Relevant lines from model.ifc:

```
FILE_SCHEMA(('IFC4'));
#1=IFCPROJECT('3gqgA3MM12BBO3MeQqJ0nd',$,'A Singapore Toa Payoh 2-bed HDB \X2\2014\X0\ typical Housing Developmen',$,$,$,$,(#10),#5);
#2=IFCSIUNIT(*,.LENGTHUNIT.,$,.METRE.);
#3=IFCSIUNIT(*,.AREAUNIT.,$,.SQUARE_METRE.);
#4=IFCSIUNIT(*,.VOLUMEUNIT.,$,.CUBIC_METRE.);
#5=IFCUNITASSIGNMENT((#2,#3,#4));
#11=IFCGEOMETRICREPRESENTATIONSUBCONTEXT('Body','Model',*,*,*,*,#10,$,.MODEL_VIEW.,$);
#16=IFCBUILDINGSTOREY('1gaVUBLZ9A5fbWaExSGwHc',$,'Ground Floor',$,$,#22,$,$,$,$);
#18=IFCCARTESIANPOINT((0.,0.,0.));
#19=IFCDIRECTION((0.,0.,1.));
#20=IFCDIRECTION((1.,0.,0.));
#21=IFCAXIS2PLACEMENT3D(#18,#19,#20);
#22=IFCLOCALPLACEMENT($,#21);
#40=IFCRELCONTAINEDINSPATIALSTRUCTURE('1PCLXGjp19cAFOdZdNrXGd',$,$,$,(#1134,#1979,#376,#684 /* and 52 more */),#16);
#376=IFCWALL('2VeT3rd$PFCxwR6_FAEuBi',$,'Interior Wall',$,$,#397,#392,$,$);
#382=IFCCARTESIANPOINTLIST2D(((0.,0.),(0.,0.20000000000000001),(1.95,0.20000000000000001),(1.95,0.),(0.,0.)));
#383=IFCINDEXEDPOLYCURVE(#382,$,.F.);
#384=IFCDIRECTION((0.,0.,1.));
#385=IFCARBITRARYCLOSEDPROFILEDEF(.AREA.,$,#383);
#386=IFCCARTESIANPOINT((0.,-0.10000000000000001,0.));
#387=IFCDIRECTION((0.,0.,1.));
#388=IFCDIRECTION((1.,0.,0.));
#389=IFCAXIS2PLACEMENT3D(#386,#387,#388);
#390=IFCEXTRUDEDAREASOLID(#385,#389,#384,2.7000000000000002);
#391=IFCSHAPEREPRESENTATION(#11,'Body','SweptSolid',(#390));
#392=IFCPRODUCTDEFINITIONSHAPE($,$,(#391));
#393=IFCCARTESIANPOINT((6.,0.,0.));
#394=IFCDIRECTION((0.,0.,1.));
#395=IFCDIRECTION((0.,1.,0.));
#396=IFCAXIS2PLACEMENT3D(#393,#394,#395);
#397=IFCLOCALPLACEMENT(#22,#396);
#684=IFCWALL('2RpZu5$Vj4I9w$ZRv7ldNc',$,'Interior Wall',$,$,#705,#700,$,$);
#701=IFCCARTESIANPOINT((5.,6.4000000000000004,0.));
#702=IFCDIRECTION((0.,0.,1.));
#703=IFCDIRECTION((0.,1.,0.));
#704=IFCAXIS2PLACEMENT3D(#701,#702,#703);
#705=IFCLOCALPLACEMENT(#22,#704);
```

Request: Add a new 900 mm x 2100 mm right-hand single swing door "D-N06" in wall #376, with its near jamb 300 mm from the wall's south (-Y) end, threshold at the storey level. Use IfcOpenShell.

```python
import numpy as np
import ifcopenshell
import ifcopenshell.api.feature
import ifcopenshell.api.geometry
import ifcopenshell.api.root
import ifcopenshell.api.spatial
import ifcopenshell.geom
import ifcopenshell.util.element
import ifcopenshell.util.placement
import ifcopenshell.util.representation
import ifcopenshell.util.shape
import ifcopenshell.util.unit

model = ifcopenshell.open("model.ifc")
unit_scale = ifcopenshell.util.unit.calculate_unit_scale(model)
settings = ifcopenshell.geom.settings()


def volume(element):
    """Net volume in cubic metres, openings subtracted."""
    shape = ifcopenshell.geom.create_shape(settings, element)
    return ifcopenshell.util.shape.get_volume(shape.geometry)


wall = model.by_guid("2VeT3rd$PFCxwR6_FAEuBi")
storey = ifcopenshell.util.element.get_container(wall, ifc_class="IfcBuildingStorey")
context = ifcopenshell.util.representation.get_context(model, "Model", "Body", "MODEL_VIEW")
before = volume(wall)

width, height, from_end, sill = 0.9, 2.1, 0.3, 0.0  # metres

# The wall runs along its own X axis, and the end named is its -X end.
wall_shape = ifcopenshell.geom.create_shape(settings, wall)
x, y, z = ifcopenshell.util.shape.get_vertices(wall_shape.geometry).T
start = x.min() + from_end
face, thickness = float(y.min()), float(y.max() - y.min())
wall_matrix = ifcopenshell.util.placement.get_local_placement(wall.ObjectPlacement)
level = ifcopenshell.util.placement.get_local_placement(storey.ObjectPlacement)[2, 3]


def in_wall(x, y):
    """Placement at x, y metres in the wall's axes, at sill height."""
    matrix = wall_matrix.copy()
    matrix[:, 3] = wall_matrix @ np.array([x / unit_scale, y / unit_scale, 0.0, 1.0])
    matrix[2, 3] = level + sill / unit_scale
    return matrix


# Opening: a box that overshoots both wall faces by 50 mm.
opening = ifcopenshell.api.root.create_entity(model, ifc_class="IfcOpeningElement", predefined_type="OPENING")
box = ifcopenshell.api.geometry.add_wall_representation(
    model, context=context, length=width, height=height, thickness=thickness + 0.1
)
ifcopenshell.api.geometry.assign_representation(model, product=opening, representation=box)
ifcopenshell.api.geometry.edit_object_placement(model, product=opening, matrix=in_wall(start, face - 0.05), is_si=False)
ifcopenshell.api.feature.add_feature(model, feature=opening, element=wall)

door = ifcopenshell.api.root.create_entity(model, ifc_class="IfcDoor", name="D-N06", predefined_type="DOOR")
door.OverallWidth, door.OverallHeight = width / unit_scale, height / unit_scale
door.OperationType = "SINGLE_SWING_RIGHT"
body = ifcopenshell.api.geometry.add_door_representation(
    model,
    context=context,
    overall_width=door.OverallWidth,
    overall_height=door.OverallHeight,
    operation_type="SINGLE_SWING_RIGHT",
    lining_properties={"LiningDepth": thickness / unit_scale, "ThresholdDepth": thickness / unit_scale},
)
ifcopenshell.api.geometry.assign_representation(model, product=door, representation=body)
ifcopenshell.api.spatial.assign_container(model, products=[door], relating_structure=storey)
ifcopenshell.api.feature.add_filling(model, opening=opening, element=door)

# The lining spans the wall, so the door starts at the wall face.
ifcopenshell.api.geometry.edit_object_placement(model, product=door, matrix=in_wall(start, face), is_si=False)

after = volume(wall)

print(f"wall volume {before:.3f} -> {after:.3f} m3")

model.write("model-out.ifc")
```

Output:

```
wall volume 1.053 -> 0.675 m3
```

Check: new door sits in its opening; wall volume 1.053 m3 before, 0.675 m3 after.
